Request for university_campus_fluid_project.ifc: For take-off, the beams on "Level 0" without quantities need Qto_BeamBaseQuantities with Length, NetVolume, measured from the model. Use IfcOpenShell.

First a look at what the model holds.

```python
import ifcopenshell
import ifcopenshell.util.element
import ifcopenshell.util.unit

model = ifcopenshell.open("university_campus_fluid_project.ifc")
print(model.schema)
for unit_type in ("LENGTHUNIT", "AREAUNIT", "VOLUMEUNIT"):
    print(unit_type, ifcopenshell.util.unit.calculate_unit_scale(model, unit_type))
storey = next(s for s in model.by_type("IfcBuildingStorey") if s.Name == "Level 0")
beams = [e for e in ifcopenshell.util.element.get_decomposition(storey) if e.is_a("IfcBeam")]
for e in sorted(beams, key=lambda e: e.id()):
    print(e.id(), e.is_a(), e.Name, list(ifcopenshell.util.element.get_psets(e, qtos_only=True)), sep=" | ")
```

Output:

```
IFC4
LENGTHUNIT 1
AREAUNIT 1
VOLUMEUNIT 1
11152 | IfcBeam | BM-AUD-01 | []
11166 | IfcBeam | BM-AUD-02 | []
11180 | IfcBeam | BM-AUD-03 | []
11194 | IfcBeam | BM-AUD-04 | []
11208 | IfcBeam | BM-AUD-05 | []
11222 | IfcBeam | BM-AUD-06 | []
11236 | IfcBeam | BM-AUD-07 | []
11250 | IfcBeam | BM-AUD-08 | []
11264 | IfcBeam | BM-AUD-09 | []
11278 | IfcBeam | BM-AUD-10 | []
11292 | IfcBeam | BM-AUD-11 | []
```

```python
import ifcopenshell
import ifcopenshell.api.pset
import ifcopenshell.geom
import ifcopenshell.util.element
import ifcopenshell.util.shape
import ifcopenshell.util.unit

model = ifcopenshell.open("university_campus_fluid_project.ifc")
unit_scale = ifcopenshell.util.unit.calculate_unit_scale(model)
volume_scale = ifcopenshell.util.unit.calculate_unit_scale(model, "VOLUMEUNIT")
settings = ifcopenshell.geom.settings()

storey = next(s for s in model.by_type("IfcBuildingStorey") if s.Name == "Level 0")
beams = [e for e in ifcopenshell.util.element.get_decomposition(storey) if e.is_a("IfcBeam")]

for e in sorted(beams, key=lambda e: e.id()):
    if ifcopenshell.util.element.get_psets(e, qtos_only=True, should_inherit=False):
        continue
    # Geometry comes back in metres, in the element's own axes.
    shape = ifcopenshell.geom.create_shape(settings, e)
    values = {
        "Length": ifcopenshell.util.shape.get_max_xyz(shape.geometry) / unit_scale,
        "NetVolume": ifcopenshell.util.shape.get_volume(shape.geometry) / volume_scale,
    }
    qto = ifcopenshell.api.pset.add_qto(model, product=e, name="Qto_BeamBaseQuantities")
    ifcopenshell.api.pset.edit_qto(model, qto=qto, properties=values)
    print(e.id(), {k: round(v, 3) for k, v in values.items()})

model.write("university_campus_fluid_project_v2.ifc")
```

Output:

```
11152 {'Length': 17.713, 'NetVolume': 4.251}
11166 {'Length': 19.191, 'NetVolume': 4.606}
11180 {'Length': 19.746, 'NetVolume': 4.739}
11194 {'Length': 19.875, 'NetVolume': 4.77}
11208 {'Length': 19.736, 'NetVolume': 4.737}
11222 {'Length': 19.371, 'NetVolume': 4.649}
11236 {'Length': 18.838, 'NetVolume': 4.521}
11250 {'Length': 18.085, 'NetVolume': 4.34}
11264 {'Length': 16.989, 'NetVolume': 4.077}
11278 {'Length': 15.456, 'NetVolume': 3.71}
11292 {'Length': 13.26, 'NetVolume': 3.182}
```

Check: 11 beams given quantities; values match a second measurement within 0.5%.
